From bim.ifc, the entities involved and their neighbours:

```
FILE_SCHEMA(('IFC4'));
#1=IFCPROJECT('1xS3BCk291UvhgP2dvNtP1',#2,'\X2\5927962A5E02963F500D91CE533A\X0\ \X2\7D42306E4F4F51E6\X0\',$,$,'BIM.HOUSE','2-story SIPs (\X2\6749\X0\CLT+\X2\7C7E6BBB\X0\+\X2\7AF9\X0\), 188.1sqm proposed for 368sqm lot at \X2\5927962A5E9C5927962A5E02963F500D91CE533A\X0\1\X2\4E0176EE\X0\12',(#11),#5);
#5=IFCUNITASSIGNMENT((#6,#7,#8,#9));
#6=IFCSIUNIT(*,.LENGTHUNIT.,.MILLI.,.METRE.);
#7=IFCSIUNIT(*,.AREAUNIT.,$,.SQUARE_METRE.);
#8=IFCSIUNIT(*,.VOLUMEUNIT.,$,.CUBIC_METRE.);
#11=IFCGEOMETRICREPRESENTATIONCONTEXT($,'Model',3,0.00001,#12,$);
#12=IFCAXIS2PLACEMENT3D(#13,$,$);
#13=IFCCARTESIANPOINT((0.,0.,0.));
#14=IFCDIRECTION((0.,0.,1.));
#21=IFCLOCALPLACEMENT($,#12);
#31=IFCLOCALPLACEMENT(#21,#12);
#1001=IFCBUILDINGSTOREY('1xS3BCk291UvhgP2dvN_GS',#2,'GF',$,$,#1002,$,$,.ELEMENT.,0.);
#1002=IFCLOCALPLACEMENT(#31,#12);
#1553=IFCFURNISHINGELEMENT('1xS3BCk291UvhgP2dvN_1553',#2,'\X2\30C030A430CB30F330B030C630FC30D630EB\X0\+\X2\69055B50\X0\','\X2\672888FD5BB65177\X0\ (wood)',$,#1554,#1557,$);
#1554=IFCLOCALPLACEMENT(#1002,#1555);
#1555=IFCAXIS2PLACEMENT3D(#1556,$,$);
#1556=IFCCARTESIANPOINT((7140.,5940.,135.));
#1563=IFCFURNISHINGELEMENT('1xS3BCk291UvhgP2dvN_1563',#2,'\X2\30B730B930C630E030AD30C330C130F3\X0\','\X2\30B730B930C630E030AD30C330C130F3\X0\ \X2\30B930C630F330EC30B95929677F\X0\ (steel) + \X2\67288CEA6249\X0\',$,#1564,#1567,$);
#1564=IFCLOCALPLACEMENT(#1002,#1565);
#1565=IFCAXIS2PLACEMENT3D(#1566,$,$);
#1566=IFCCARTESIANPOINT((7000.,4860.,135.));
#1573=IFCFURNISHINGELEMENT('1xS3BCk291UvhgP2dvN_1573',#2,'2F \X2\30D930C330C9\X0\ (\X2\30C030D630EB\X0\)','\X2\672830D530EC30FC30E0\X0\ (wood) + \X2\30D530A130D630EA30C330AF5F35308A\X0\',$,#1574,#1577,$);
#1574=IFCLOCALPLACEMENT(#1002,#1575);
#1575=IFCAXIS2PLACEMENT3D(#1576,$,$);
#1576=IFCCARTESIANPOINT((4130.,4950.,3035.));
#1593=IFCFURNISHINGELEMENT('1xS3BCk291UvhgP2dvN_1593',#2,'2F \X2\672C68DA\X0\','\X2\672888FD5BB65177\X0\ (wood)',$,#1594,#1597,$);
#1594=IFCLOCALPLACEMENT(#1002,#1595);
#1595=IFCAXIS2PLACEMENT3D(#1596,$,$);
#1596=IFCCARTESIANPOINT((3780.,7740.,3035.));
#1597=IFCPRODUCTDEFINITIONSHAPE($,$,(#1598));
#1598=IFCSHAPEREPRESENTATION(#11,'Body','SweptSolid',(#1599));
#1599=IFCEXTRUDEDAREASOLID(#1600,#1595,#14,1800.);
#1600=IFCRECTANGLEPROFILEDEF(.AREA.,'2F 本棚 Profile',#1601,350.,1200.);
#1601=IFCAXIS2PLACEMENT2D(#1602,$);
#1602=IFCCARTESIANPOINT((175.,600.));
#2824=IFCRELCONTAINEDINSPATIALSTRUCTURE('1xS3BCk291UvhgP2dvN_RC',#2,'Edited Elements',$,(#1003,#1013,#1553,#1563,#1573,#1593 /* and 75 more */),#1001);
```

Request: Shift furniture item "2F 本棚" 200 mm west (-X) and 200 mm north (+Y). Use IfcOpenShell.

```python
import ifcopenshell
import ifcopenshell.api.geometry
import ifcopenshell.util.placement

model = ifcopenshell.open("bim.ifc")

item = model.by_guid("1xS3BCk291UvhgP2dvN_1593")
matrix = ifcopenshell.util.placement.get_local_placement(item.ObjectPlacement)
matrix[0, 3] -= 200.0
matrix[1, 3] += 200.0
ifcopenshell.api.geometry.edit_object_placement(model, product=item, matrix=matrix, is_si=False)

print(ifcopenshell.util.placement.get_local_placement(item.ObjectPlacement).round(3) + 0.0)

model.write("bim_rev.ifc")
```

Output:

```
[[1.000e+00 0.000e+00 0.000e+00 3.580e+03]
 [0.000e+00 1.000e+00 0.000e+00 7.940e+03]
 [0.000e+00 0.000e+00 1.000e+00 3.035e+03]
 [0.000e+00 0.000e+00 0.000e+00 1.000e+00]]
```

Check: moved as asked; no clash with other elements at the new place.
